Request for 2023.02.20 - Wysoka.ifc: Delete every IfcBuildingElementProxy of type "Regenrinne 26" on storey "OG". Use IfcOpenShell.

First a look at what the model holds.

```python
import ifcopenshell
import ifcopenshell.util.element

model = ifcopenshell.open("2023.02.20 - Wysoka.ifc")
print(model.schema)
storey = next(s for s in model.by_type("IfcBuildingStorey") if s.Name == "OG")
proxies = [e for e in ifcopenshell.util.element.get_decomposition(storey) if e.is_a("IfcBuildingElementProxy")]
seen = {}
for e in proxies:
    element_type = ifcopenshell.util.element.get_type(e)
    name = element_type.Name if element_type not in (None, e) else None
    seen[name] = seen.get(name, 0) + 1
for name, count in sorted(seen.items(), key=str):
    print(count, "x", name)
```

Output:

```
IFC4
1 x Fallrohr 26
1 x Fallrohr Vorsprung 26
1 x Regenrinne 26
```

```python
import ifcopenshell
import ifcopenshell.api.root
import ifcopenshell.util.element

model = ifcopenshell.open("2023.02.20 - Wysoka.ifc")

storey = next(s for s in model.by_type("IfcBuildingStorey") if s.Name == "OG")
proxies = [e for e in ifcopenshell.util.element.get_decomposition(storey) if e.is_a("IfcBuildingElementProxy")]
targets = [e for e in proxies if (t := ifcopenshell.util.element.get_type(e)) not in (None, e) and t.Name == "Regenrinne 26"]

for e in targets:
    ifcopenshell.api.root.remove_product(model, product=e)
print(len(targets), "removed")

model.write("2023.02.20 - Wysoka_edited.ifc")
```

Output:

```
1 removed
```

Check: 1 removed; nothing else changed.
